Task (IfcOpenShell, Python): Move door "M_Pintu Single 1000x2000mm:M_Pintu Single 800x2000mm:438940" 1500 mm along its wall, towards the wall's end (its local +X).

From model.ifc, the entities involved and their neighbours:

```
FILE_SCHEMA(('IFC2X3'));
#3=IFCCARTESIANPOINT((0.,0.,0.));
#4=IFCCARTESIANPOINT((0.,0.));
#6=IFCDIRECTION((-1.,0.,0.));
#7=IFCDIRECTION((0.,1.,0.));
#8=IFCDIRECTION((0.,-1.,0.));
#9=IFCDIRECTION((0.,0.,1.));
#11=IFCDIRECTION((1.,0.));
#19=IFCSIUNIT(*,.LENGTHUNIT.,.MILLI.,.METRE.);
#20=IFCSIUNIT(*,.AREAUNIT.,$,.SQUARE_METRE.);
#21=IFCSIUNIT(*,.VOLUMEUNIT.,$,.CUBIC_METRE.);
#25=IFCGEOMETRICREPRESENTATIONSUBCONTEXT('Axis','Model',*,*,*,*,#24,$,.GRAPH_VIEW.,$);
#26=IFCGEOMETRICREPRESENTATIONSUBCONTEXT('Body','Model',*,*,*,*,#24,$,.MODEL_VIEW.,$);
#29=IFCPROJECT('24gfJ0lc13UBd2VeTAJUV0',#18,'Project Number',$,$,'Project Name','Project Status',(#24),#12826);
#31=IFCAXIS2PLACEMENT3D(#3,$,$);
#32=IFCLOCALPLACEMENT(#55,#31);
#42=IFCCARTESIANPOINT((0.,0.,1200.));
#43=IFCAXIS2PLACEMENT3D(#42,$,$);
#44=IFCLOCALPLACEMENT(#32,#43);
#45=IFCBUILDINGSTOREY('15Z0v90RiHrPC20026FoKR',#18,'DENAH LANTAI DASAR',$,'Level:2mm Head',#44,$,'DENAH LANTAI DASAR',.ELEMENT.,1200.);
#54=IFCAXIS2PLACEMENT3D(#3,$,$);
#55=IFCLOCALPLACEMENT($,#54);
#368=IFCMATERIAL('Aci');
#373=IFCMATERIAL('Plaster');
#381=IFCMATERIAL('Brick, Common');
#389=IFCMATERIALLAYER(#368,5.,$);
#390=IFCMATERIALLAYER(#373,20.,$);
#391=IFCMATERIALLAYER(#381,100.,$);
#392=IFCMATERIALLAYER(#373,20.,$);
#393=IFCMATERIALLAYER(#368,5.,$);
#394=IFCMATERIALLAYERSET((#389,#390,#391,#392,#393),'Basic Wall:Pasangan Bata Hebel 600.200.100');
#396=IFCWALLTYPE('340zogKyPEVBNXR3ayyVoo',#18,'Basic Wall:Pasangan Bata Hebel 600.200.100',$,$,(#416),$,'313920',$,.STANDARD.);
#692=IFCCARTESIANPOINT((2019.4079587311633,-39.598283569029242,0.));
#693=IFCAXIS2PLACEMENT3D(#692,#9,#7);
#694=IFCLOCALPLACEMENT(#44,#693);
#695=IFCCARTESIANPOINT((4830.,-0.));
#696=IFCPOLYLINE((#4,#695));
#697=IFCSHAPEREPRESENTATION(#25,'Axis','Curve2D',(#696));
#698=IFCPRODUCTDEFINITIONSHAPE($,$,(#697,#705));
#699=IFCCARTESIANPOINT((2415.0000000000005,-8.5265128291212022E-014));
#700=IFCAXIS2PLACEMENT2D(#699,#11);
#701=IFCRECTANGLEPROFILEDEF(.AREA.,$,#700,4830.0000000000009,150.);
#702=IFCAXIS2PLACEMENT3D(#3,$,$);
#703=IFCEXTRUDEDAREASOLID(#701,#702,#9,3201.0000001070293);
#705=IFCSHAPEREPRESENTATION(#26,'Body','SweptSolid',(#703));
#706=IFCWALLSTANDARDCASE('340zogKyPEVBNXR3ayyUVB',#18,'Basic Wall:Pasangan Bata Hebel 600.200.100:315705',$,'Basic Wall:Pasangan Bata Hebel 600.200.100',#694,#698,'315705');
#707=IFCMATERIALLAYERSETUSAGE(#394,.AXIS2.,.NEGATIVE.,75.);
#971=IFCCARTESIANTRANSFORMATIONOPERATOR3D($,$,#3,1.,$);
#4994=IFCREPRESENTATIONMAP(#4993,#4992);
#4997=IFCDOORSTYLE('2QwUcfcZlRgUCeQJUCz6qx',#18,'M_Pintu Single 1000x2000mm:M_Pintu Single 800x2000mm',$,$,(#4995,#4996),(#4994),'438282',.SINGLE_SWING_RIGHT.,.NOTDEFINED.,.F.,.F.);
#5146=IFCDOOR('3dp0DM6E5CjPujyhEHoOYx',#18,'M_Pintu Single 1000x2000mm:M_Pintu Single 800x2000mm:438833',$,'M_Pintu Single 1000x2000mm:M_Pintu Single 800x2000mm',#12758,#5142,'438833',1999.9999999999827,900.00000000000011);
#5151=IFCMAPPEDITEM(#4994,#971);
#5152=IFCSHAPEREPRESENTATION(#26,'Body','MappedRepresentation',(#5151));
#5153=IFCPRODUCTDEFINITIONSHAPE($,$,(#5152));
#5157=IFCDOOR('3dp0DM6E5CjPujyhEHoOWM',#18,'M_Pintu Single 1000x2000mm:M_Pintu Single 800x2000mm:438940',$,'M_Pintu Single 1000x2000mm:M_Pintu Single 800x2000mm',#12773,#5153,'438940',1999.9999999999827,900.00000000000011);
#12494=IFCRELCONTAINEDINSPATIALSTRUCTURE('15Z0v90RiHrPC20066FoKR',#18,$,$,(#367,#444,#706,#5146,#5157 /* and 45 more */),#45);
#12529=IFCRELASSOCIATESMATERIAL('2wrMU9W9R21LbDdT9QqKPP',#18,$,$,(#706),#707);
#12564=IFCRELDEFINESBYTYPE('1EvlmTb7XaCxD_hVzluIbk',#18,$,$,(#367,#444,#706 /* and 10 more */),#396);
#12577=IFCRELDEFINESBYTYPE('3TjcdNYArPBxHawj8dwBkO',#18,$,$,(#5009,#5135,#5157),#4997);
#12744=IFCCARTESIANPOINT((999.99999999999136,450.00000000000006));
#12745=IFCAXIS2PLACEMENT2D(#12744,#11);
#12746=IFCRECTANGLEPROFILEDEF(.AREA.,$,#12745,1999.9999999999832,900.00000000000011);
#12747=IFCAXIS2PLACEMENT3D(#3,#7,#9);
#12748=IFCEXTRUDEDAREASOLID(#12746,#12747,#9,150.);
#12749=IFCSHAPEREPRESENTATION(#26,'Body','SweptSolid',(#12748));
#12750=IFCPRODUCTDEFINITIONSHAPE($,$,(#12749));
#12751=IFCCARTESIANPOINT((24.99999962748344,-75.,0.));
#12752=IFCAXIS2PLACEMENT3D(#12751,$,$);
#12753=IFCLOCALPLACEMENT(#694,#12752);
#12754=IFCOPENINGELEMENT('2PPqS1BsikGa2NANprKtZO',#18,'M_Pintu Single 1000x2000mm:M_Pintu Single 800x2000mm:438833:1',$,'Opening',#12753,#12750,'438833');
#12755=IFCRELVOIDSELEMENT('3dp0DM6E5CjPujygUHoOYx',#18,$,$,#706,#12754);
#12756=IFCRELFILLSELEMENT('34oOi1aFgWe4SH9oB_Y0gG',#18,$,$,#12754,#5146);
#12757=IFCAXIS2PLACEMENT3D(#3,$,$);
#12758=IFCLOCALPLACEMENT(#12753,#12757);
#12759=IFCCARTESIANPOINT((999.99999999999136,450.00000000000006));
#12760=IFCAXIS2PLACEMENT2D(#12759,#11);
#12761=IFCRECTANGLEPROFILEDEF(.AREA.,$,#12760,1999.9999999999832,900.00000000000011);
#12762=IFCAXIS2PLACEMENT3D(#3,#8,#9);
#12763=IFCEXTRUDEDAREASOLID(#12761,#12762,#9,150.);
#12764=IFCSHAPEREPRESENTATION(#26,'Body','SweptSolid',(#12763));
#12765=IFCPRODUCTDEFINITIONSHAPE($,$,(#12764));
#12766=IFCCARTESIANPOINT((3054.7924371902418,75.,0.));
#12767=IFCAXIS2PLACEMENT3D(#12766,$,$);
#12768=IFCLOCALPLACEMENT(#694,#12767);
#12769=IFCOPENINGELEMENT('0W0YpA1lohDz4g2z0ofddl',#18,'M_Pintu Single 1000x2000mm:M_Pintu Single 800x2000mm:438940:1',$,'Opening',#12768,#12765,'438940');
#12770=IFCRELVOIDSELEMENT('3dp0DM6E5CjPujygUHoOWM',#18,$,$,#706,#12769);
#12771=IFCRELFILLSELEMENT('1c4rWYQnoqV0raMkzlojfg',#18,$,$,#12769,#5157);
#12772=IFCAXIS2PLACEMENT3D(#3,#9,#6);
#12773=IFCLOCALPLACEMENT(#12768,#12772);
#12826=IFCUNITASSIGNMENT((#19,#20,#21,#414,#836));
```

```python
import ifcopenshell
import ifcopenshell.api.geometry
import ifcopenshell.util.placement

model = ifcopenshell.open("model.ifc")

door = model.by_id(5157)
opening = door.FillsVoids[0].RelatingOpeningElement
wall = opening.VoidsElements[0].RelatingBuildingElement

wall_matrix = ifcopenshell.util.placement.get_local_placement(wall.ObjectPlacement)
shift = wall_matrix[:3, 0] * 1500.0
before = ifcopenshell.util.placement.get_local_placement(door.ObjectPlacement)[:3, 3].copy()

# The door is placed relative to its opening, so it follows when the opening moves.
matrix = ifcopenshell.util.placement.get_local_placement(opening.ObjectPlacement)
matrix[:3, 3] += shift
ifcopenshell.api.geometry.edit_object_placement(
    model, product=opening, matrix=matrix, is_si=False, should_transform_children=True
)

after = ifcopenshell.util.placement.get_local_placement(door.ObjectPlacement)[:3, 3]
print("door moved by", (after - before).round(3) + 0.0)

model.write("model_edited.ifc")
```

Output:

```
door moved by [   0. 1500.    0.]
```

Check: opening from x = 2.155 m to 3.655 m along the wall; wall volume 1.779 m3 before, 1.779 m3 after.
